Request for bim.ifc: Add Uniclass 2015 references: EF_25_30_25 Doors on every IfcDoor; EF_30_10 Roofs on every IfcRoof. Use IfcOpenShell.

First a look at what the model holds.

```python
import ifcopenshell

model = ifcopenshell.open("bim.ifc")
print(model.schema)
print("classifications:", [c.Name for c in model.by_type("IfcClassification")])
for ifc_class in ("IfcDoor", "IfcRoof", "IfcStair", "IfcWall", "IfcWindow"):
    print(ifc_class, len(model.by_type(ifc_class)))
```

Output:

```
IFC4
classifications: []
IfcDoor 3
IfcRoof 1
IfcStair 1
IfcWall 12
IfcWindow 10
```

```python
import ifcopenshell
import ifcopenshell.api.classification

model = ifcopenshell.open("bim.ifc")

system = ifcopenshell.api.classification.add_classification(model, classification="Uniclass 2015")

codes = {
    "IfcDoor": ("EF_25_30_25", "Doors"),
    "IfcRoof": ("EF_30_10", "Roofs"),
}
for ifc_class, (code, name) in codes.items():
    products = model.by_type(ifc_class)
    ifcopenshell.api.classification.add_reference(
        model, products=products, classification=system, identification=code, name=name
    )
    print(code, len(products))

model.write("bim_rev.ifc")
```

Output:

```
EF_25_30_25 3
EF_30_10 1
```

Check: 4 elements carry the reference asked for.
